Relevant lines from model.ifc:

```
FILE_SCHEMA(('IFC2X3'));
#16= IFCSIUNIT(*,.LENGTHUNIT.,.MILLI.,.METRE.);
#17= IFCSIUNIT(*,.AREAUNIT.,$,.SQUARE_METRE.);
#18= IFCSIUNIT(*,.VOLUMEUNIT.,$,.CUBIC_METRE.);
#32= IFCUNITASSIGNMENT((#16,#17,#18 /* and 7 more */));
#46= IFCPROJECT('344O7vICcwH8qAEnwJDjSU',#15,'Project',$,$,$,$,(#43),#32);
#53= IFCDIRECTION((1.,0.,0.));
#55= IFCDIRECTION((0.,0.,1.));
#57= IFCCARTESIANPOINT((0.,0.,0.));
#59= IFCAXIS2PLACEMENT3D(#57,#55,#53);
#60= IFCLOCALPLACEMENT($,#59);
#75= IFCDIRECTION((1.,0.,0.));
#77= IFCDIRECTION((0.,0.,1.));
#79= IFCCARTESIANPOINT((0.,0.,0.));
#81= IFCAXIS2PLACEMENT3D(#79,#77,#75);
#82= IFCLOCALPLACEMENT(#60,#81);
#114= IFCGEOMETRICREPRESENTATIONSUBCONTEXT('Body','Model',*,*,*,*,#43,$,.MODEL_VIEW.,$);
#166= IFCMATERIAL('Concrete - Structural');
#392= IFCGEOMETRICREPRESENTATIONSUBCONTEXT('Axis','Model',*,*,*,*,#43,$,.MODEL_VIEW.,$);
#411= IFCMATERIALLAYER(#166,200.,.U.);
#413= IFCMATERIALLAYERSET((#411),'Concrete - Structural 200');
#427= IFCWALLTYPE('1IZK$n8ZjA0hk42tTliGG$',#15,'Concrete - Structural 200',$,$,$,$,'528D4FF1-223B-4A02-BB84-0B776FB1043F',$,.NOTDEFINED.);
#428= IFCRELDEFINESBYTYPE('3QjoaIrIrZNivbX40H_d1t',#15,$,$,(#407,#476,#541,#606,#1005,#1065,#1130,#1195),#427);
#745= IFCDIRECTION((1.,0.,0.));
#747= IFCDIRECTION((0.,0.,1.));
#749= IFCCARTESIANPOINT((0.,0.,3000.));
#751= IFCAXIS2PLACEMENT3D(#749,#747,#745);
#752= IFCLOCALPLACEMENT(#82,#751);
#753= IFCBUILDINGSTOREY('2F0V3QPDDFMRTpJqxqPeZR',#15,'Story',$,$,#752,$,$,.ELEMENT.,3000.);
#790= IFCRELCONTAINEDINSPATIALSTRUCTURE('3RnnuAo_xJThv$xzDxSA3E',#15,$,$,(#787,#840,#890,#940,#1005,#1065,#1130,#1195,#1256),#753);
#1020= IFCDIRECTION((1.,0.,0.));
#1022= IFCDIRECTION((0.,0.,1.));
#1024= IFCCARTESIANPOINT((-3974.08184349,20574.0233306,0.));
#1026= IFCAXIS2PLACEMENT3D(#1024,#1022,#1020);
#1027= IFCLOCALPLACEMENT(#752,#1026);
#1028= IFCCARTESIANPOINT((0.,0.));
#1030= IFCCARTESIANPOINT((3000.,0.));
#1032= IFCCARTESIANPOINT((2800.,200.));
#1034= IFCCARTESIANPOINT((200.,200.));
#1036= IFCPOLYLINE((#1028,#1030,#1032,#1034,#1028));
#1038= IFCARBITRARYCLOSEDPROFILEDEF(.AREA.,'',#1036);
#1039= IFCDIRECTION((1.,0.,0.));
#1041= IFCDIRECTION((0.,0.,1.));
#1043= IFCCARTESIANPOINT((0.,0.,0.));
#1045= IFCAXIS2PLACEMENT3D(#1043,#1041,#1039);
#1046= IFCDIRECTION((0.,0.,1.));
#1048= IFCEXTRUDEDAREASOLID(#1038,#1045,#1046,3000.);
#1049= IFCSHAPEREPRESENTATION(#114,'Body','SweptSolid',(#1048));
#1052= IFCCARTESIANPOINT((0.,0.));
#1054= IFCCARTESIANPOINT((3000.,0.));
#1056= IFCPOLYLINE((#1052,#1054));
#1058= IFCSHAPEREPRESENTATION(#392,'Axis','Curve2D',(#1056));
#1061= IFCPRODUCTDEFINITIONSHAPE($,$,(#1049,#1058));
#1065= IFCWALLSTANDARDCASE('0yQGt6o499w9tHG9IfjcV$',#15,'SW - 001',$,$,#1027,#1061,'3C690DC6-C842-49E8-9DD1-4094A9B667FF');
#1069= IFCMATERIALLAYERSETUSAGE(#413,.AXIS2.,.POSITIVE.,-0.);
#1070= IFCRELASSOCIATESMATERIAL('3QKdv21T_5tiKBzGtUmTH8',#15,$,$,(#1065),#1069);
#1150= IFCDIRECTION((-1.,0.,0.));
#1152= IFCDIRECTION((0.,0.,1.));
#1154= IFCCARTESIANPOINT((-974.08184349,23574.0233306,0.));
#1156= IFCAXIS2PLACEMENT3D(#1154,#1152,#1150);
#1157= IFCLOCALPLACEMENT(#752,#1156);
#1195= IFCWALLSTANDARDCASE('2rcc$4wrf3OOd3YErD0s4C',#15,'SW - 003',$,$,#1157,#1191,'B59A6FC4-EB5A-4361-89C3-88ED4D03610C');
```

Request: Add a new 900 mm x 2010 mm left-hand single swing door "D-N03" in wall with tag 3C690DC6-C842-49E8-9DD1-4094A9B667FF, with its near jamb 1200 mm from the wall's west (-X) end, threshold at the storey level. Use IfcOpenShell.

```python
import numpy as np
import ifcopenshell
import ifcopenshell.api.feature
import ifcopenshell.api.geometry
import ifcopenshell.api.root
import ifcopenshell.api.spatial
import ifcopenshell.api.type
import ifcopenshell.geom
import ifcopenshell.util.element
import ifcopenshell.util.placement
import ifcopenshell.util.representation
import ifcopenshell.util.shape
import ifcopenshell.util.unit

model = ifcopenshell.open("model.ifc")
unit_scale = ifcopenshell.util.unit.calculate_unit_scale(model)
settings = ifcopenshell.geom.settings()


def volume(element):
    """Net volume in cubic metres, openings subtracted."""
    shape = ifcopenshell.geom.create_shape(settings, element)
    return ifcopenshell.util.shape.get_volume(shape.geometry)


wall = model.by_guid("0yQGt6o499w9tHG9IfjcV$")
storey = ifcopenshell.util.element.get_container(wall, ifc_class="IfcBuildingStorey")
context = ifcopenshell.util.representation.get_context(model, "Model", "Body", "MODEL_VIEW")
before = volume(wall)

width, height, from_end, sill = 0.9, 2.01, 1.2, 0.0  # metres

# The wall runs along its own X axis, and the end named is its -X end.
wall_shape = ifcopenshell.geom.create_shape(settings, wall)
x, y, z = ifcopenshell.util.shape.get_vertices(wall_shape.geometry).T
start = x.min() + from_end
face, thickness = float(y.min()), float(y.max() - y.min())
wall_matrix = ifcopenshell.util.placement.get_local_placement(wall.ObjectPlacement)
level = ifcopenshell.util.placement.get_local_placement(storey.ObjectPlacement)[2, 3]


def in_wall(x, y):
    """Placement at x, y metres in the wall's axes, at sill height."""
    matrix = wall_matrix.copy()
    matrix[:, 3] = wall_matrix @ np.array([x / unit_scale, y / unit_scale, 0.0, 1.0])
    matrix[2, 3] = level + sill / unit_scale
    return matrix


# Opening: a box that overshoots both wall faces by 50 mm.
opening = ifcopenshell.api.root.create_entity(model, ifc_class="IfcOpeningElement")
box = ifcopenshell.api.geometry.add_wall_representation(
    model, context=context, length=width, height=height, thickness=thickness + 0.1
)
ifcopenshell.api.geometry.assign_representation(model, product=opening, representation=box)
ifcopenshell.api.geometry.edit_object_placement(model, product=opening, matrix=in_wall(start, face - 0.05), is_si=False)
ifcopenshell.api.feature.add_feature(model, feature=opening, element=wall)

door = ifcopenshell.api.root.create_entity(model, ifc_class="IfcDoor", name="D-N03")
door.OverallWidth, door.OverallHeight = width / unit_scale, height / unit_scale
body = ifcopenshell.api.geometry.add_door_representation(
    model,
    context=context,
    overall_width=door.OverallWidth,
    overall_height=door.OverallHeight,
    operation_type="SINGLE_SWING_LEFT",
    lining_properties={"LiningDepth": thickness / unit_scale, "ThresholdDepth": thickness / unit_scale},
)
ifcopenshell.api.geometry.assign_representation(model, product=door, representation=body)
ifcopenshell.api.spatial.assign_container(model, products=[door], relating_structure=storey)
fills = ifcopenshell.api.feature.add_filling(model, opening=opening, element=door)
fills.OwnerHistory = door.OwnerHistory  # required in IFC2X3

# IFC2X3 keeps the operation on the door style.
style = ifcopenshell.api.root.create_entity(model, ifc_class="IfcDoorStyle", name="D-N03")
style.OperationType, style.ConstructionType = "SINGLE_SWING_LEFT", "NOTDEFINED"
style.ParameterTakesPrecedence = style.Sizeable = False
ifcopenshell.api.type.assign_type(model, related_objects=[door], relating_type=style)

# The lining spans the wall, so the door starts at the wall face.
ifcopenshell.api.geometry.edit_object_placement(model, product=door, matrix=in_wall(start, face), is_si=False)

after = volume(wall)

print(f"wall volume {before:.3f} -> {after:.3f} m3")

model.write("model_rev.ifc")
```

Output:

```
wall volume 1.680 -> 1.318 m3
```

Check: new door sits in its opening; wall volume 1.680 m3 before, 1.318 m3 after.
